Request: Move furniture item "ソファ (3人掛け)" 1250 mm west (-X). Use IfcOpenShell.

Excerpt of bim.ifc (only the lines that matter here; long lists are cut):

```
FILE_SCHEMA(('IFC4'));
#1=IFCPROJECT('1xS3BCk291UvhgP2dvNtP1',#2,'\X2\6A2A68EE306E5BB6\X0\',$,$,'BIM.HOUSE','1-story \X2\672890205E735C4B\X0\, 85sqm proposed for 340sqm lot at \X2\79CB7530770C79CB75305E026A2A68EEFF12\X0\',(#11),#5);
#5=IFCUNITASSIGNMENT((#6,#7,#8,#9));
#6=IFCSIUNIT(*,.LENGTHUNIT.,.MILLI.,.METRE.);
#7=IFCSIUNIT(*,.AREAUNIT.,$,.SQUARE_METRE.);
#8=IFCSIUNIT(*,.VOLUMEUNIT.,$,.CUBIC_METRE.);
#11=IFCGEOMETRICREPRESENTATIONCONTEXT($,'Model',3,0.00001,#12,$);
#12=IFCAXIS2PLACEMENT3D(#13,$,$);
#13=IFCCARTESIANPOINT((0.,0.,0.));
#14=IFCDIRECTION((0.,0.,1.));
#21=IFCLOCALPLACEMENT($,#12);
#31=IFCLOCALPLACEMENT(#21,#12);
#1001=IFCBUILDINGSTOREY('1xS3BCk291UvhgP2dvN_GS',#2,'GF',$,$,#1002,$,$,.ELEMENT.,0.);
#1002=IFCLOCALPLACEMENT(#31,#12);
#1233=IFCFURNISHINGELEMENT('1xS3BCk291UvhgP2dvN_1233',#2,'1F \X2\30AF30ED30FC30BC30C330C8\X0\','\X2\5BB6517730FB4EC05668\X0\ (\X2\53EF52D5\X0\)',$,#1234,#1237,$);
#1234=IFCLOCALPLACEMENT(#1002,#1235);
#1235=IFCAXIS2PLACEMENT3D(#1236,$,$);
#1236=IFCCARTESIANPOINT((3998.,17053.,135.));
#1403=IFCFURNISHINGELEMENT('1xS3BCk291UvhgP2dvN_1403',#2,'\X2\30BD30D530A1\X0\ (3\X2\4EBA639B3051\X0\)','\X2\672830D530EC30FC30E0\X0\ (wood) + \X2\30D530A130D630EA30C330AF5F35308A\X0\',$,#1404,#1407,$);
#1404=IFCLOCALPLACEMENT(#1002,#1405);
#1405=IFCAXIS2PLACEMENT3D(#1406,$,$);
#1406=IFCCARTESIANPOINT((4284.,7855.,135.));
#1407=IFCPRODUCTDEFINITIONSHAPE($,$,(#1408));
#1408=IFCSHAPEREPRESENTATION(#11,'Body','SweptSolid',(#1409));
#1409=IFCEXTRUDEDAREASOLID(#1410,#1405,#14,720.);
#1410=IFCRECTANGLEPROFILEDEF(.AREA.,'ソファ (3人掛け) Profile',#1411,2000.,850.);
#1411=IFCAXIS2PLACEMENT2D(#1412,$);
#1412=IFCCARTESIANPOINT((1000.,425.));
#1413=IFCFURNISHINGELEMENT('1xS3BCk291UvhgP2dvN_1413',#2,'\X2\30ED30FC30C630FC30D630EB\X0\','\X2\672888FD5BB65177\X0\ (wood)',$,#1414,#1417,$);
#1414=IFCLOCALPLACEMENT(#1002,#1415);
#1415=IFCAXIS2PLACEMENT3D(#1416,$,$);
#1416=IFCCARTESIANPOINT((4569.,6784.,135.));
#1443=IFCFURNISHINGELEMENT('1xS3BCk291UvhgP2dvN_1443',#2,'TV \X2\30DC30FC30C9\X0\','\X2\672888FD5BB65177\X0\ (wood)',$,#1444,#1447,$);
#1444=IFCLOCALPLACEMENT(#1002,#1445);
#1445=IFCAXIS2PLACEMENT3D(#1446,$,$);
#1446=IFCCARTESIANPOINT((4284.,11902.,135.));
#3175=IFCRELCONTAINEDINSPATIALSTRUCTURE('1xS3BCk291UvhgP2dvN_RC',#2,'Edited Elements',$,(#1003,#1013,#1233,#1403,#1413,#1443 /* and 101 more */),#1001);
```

```python
import ifcopenshell
import ifcopenshell.api.geometry
import ifcopenshell.util.placement
import ifcopenshell.util.unit

model = ifcopenshell.open("bim.ifc")
unit_scale = ifcopenshell.util.unit.calculate_unit_scale(model)

item = model.by_guid("1xS3BCk291UvhgP2dvN_1403")
matrix = ifcopenshell.util.placement.get_local_placement(item.ObjectPlacement)
matrix[0, 3] -= 1.25 / unit_scale
ifcopenshell.api.geometry.edit_object_placement(model, product=item, matrix=matrix, is_si=False)

print(ifcopenshell.util.placement.get_local_placement(item.ObjectPlacement).round(3) + 0.0)

model.write("bim_edited.ifc")
```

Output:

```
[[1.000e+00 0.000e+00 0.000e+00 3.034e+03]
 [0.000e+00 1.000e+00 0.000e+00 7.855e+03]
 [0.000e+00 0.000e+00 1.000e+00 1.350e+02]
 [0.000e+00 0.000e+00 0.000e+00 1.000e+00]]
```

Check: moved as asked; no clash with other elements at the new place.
